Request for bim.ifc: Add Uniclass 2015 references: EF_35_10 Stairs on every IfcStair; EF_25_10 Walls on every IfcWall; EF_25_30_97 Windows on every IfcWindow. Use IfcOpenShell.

First a look at what the model holds.

```python
import ifcopenshell

model = ifcopenshell.open("bim.ifc")
print(model.schema)
print("classifications:", [c.Name for c in model.by_type("IfcClassification")])
for ifc_class in ("IfcDoor", "IfcRoof", "IfcStair", "IfcWall", "IfcWindow"):
    print(ifc_class, len(model.by_type(ifc_class)))
```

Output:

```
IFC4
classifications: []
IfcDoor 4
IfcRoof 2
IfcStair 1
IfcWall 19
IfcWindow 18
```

```python
import ifcopenshell
import ifcopenshell.api.classification

model = ifcopenshell.open("bim.ifc")

system = ifcopenshell.api.classification.add_classification(model, classification="Uniclass 2015")

codes = {
    "IfcStair": ("EF_35_10", "Stairs"),
    "IfcWall": ("EF_25_10", "Walls"),
    "IfcWindow": ("EF_25_30_97", "Windows"),
}
for ifc_class, (code, name) in codes.items():
    products = model.by_type(ifc_class)
    ifcopenshell.api.classification.add_reference(
        model, products=products, classification=system, identification=code, name=name
    )
    print(code, len(products))

model.write("bim_v2.ifc")
```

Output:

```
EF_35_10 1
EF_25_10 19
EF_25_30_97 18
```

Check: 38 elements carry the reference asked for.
